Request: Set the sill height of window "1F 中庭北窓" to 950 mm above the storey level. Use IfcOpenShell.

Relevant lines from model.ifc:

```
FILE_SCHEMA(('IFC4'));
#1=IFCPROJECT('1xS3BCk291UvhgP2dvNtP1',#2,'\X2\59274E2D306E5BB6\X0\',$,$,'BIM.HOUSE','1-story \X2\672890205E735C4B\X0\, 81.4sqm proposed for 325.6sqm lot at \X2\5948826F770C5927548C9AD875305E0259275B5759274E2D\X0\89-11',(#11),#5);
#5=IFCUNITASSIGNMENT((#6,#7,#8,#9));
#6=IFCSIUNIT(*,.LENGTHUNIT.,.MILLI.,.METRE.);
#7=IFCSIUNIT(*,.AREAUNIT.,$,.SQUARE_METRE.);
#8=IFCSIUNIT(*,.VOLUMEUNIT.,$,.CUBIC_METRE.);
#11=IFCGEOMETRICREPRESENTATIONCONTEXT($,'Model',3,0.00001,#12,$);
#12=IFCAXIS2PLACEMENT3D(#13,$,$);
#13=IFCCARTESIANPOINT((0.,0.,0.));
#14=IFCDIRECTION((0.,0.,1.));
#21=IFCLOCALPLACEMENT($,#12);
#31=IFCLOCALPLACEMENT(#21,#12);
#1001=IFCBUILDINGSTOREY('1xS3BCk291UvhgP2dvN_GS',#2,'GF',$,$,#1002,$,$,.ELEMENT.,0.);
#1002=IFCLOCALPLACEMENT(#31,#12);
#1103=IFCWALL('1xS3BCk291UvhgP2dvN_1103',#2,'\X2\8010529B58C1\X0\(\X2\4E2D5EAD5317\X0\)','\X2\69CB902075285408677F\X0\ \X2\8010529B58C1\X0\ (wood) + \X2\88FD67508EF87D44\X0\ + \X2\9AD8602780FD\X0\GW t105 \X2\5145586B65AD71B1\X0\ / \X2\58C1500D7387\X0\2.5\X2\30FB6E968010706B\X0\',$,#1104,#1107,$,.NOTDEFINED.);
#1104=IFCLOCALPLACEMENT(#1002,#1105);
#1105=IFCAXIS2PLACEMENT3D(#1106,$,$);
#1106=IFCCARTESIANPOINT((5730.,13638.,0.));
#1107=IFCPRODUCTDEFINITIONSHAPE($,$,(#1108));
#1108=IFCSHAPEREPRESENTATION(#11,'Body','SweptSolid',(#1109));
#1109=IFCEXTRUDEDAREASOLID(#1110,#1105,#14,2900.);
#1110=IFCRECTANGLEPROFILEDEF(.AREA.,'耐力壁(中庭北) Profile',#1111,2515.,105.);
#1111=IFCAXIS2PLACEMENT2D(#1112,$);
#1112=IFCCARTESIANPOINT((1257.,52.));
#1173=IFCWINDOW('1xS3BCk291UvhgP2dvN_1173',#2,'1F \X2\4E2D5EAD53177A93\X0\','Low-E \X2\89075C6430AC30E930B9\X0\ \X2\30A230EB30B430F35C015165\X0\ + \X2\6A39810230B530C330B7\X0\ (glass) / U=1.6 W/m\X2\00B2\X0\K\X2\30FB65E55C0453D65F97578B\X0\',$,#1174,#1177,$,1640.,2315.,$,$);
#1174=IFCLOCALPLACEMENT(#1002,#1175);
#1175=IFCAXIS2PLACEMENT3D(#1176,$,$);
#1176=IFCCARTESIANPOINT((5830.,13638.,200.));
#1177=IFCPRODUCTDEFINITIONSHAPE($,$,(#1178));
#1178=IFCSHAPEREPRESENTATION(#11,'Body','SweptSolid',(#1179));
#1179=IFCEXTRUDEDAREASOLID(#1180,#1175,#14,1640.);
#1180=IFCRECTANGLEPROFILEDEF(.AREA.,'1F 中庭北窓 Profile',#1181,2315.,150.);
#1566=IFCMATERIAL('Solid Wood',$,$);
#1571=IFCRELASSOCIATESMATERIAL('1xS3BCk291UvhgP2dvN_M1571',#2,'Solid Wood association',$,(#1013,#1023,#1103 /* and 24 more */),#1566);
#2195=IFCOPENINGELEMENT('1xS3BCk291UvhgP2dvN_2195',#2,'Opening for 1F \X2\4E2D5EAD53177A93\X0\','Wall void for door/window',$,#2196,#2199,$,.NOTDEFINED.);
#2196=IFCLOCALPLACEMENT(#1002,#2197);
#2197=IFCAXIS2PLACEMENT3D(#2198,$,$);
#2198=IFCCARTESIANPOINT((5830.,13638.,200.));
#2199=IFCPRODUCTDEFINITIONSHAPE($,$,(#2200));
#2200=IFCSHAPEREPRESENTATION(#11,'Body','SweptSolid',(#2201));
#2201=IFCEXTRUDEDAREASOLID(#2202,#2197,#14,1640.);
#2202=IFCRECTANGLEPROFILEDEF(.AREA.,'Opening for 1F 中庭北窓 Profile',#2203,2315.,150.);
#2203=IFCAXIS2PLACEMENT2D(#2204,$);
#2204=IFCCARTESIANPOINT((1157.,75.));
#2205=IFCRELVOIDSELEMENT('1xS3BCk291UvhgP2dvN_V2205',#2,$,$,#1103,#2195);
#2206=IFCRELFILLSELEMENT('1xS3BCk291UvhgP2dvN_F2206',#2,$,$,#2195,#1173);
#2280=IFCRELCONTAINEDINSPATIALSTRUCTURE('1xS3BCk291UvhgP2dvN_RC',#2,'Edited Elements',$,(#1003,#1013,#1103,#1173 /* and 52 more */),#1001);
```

```python
import numpy as np
import ifcopenshell
import ifcopenshell.api.geometry
import ifcopenshell.geom
import ifcopenshell.util.element
import ifcopenshell.util.placement
import ifcopenshell.util.shape
import ifcopenshell.util.unit

model = ifcopenshell.open("model.ifc")
unit_scale = ifcopenshell.util.unit.calculate_unit_scale(model)

window = model.by_guid("1xS3BCk291UvhgP2dvN_1173")
opening = window.FillsVoids[0].RelatingOpeningElement
storey = ifcopenshell.util.element.get_container(window, ifc_class="IfcBuildingStorey")
level = ifcopenshell.util.placement.get_local_placement(storey.ObjectPlacement)[2, 3]

# The opening's origin need not be at the sill, so measure its lowest point.
shape = ifcopenshell.geom.create_shape(ifcopenshell.geom.settings(), opening)
bottom = ifcopenshell.util.shape.get_shape_bottom_elevation(shape, shape.geometry) / unit_scale
dz = level + 950.0 - bottom

shift = np.array([0.0, 0.0, dz])
# The window is not placed relative to its opening, so move both.
for product in (opening, window):
    matrix = ifcopenshell.util.placement.get_local_placement(product.ObjectPlacement)
    matrix[:3, 3] += shift
    ifcopenshell.api.geometry.edit_object_placement(model, product=product, matrix=matrix, is_si=False)

print(f"moved by {dz * unit_scale:+.3f} m")

model.write("model_updated.ifc")
```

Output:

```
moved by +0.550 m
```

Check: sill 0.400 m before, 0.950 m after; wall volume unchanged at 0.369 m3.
